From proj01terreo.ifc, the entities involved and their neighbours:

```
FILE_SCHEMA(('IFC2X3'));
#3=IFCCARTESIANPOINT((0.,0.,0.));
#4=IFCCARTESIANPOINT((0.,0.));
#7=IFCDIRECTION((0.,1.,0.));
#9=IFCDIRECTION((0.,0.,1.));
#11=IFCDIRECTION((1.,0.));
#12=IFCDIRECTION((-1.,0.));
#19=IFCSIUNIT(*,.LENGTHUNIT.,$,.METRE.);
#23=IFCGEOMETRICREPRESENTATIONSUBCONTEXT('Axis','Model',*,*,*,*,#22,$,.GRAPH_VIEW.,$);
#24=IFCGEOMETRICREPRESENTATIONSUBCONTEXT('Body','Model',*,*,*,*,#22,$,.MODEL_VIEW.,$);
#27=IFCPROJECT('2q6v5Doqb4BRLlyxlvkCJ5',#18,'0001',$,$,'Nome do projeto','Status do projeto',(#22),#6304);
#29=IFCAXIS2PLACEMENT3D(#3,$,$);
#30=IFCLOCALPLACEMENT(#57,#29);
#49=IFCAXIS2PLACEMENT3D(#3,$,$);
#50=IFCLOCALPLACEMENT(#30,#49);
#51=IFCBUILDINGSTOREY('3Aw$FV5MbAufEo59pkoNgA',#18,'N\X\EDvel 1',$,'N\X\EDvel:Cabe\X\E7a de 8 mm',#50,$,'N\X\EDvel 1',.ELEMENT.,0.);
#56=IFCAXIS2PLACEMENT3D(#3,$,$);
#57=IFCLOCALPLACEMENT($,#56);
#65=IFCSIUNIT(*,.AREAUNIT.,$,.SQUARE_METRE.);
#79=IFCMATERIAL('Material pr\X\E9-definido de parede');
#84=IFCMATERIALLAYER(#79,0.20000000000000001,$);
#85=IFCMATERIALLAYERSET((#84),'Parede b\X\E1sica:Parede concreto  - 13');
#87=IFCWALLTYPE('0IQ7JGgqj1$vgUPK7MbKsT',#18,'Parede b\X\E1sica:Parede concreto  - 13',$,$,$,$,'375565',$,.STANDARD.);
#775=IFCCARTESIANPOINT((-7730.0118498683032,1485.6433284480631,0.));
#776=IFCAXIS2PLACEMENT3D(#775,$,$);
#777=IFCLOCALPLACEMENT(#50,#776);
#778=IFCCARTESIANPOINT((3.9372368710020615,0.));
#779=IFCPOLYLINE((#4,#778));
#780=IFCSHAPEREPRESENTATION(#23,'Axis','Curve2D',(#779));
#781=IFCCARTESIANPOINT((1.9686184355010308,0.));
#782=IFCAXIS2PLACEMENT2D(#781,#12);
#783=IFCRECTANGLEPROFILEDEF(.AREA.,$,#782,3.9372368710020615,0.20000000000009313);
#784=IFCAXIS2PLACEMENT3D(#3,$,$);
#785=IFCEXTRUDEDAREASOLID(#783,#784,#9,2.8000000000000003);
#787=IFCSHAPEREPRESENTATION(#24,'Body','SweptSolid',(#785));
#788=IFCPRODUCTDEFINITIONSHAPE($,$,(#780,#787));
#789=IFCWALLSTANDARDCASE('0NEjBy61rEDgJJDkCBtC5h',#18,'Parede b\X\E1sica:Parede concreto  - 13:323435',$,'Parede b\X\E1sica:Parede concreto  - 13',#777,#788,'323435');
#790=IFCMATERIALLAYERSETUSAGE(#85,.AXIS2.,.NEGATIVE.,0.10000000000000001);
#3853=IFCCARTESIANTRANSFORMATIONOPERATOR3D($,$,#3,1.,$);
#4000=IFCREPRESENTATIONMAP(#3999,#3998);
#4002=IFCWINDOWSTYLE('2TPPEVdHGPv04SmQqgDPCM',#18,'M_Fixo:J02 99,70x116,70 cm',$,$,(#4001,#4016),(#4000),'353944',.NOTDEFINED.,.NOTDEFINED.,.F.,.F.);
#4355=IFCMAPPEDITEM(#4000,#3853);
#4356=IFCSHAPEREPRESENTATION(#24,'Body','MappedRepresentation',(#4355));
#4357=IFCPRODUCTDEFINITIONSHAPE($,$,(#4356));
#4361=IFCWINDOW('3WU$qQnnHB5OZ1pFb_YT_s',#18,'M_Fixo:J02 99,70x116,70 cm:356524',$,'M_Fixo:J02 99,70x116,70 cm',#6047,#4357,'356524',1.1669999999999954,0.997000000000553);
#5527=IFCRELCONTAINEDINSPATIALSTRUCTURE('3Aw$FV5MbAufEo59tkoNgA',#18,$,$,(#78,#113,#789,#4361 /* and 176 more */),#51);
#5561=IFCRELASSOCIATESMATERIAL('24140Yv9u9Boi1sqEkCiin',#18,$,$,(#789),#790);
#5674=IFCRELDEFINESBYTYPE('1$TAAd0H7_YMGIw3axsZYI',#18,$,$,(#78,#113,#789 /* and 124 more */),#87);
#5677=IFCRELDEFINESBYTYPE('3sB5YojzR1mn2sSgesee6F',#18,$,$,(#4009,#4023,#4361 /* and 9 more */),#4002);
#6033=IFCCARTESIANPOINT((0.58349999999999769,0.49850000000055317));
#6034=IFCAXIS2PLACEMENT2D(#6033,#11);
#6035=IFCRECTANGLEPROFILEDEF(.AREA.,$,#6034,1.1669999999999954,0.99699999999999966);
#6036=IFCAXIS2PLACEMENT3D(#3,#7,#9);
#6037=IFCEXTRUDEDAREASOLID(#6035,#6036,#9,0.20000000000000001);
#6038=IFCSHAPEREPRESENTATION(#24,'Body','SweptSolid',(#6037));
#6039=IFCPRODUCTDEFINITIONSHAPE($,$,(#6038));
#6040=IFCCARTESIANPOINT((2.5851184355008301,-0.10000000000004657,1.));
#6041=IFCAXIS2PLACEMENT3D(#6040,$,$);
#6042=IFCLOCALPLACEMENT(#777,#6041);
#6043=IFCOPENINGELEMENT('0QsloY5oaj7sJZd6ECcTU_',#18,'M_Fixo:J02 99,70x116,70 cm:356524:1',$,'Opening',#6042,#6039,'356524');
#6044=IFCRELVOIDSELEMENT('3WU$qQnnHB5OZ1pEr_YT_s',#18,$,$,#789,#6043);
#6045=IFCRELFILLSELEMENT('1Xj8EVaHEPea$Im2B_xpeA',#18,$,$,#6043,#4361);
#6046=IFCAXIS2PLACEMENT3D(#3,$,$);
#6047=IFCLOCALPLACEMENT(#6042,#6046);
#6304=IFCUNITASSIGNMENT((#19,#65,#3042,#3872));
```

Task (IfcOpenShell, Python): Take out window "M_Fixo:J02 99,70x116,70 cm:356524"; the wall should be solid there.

```python
import ifcopenshell
import ifcopenshell.api.feature
import ifcopenshell.api.root
import ifcopenshell.geom
import ifcopenshell.util.shape

model = ifcopenshell.open("proj01terreo.ifc")
settings = ifcopenshell.geom.settings()


def volume(element):
    """Net volume in cubic metres, openings subtracted."""
    shape = ifcopenshell.geom.create_shape(settings, element)
    return ifcopenshell.util.shape.get_volume(shape.geometry)


window = model.by_guid("3WU$qQnnHB5OZ1pFb_YT_s")
opening = window.FillsVoids[0].RelatingOpeningElement
wall = opening.VoidsElements[0].RelatingBuildingElement
before = volume(wall)

ifcopenshell.api.root.remove_product(model, product=window)
ifcopenshell.api.feature.remove_feature(model, feature=opening)

after = volume(wall)

print(f"wall volume {before:.3f} -> {after:.3f} m3")

model.write("proj01terreo_updated.ifc")
```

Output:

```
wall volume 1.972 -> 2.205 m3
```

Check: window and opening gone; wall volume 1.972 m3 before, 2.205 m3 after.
